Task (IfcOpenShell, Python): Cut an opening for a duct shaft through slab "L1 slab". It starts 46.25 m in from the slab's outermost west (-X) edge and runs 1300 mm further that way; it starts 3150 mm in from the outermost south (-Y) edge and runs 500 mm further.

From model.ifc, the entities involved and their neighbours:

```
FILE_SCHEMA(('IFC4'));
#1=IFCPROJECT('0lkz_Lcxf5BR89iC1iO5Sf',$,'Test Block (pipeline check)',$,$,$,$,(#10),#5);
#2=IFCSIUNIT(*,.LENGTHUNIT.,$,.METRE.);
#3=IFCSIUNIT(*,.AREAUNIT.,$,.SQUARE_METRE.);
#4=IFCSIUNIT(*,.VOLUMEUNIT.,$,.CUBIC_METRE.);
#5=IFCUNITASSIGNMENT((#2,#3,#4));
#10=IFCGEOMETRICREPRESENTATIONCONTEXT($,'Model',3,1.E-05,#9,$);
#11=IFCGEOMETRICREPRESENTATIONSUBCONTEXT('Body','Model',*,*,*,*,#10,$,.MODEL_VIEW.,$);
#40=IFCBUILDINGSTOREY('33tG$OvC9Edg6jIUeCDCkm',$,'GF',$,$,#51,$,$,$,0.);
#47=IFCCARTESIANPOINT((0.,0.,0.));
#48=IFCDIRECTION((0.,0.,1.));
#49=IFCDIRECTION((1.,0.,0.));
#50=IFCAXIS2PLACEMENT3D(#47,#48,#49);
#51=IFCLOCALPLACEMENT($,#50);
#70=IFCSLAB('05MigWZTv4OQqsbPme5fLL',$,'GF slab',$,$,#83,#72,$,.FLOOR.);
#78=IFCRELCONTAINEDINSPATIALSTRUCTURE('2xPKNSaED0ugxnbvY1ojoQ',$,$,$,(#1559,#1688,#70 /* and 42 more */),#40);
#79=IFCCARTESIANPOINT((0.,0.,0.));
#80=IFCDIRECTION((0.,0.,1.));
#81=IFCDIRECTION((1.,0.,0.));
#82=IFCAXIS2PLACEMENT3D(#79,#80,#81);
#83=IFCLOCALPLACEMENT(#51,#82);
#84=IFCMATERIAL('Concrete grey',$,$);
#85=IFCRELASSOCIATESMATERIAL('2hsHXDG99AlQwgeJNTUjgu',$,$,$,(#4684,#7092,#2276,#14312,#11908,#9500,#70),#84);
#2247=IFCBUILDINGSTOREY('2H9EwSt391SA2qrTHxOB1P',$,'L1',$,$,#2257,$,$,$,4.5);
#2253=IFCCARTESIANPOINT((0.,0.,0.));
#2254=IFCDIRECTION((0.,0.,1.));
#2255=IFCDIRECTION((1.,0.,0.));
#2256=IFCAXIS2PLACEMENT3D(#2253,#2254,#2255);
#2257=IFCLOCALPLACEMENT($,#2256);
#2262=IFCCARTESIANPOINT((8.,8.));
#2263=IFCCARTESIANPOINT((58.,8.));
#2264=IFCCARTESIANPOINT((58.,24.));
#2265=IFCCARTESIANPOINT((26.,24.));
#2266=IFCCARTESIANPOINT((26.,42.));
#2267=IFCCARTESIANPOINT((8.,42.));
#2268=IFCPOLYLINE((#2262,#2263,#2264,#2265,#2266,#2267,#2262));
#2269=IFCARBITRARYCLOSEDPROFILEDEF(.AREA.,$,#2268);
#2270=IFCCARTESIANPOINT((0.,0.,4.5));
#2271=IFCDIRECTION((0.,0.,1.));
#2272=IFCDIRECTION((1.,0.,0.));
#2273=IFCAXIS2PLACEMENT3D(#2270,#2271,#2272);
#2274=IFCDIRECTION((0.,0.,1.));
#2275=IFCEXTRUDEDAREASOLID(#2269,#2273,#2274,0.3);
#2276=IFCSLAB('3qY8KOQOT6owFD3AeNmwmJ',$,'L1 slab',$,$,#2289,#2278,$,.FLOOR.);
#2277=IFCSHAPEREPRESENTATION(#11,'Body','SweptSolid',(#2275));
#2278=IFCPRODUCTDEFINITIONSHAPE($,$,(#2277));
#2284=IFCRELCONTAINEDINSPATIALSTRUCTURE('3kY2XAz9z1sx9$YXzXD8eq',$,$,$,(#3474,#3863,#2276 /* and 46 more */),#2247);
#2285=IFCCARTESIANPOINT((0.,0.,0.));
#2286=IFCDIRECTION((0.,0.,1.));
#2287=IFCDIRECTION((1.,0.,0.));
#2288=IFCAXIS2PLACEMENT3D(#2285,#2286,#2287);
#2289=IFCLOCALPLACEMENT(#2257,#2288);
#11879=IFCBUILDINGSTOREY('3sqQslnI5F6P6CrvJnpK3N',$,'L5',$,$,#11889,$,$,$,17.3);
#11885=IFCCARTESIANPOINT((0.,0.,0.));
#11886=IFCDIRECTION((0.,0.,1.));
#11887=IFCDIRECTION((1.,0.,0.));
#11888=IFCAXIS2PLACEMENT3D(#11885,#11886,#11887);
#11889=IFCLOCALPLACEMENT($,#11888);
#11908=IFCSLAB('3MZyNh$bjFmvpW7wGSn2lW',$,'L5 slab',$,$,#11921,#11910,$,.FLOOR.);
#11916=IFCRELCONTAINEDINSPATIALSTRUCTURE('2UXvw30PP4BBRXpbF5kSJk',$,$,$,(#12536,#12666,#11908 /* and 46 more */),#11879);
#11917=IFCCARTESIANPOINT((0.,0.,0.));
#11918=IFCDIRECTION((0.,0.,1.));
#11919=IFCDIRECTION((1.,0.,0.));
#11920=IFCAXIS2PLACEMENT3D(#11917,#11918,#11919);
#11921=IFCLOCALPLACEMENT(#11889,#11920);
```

```python
import numpy as np
import ifcopenshell
import ifcopenshell.api.feature
import ifcopenshell.api.geometry
import ifcopenshell.api.root
import ifcopenshell.geom
import ifcopenshell.util.placement
import ifcopenshell.util.representation
import ifcopenshell.util.shape
import ifcopenshell.util.unit

model = ifcopenshell.open("model.ifc")
unit_scale = ifcopenshell.util.unit.calculate_unit_scale(model)
settings = ifcopenshell.geom.settings()


def volume(element):
    """Net volume in cubic metres, openings subtracted."""
    shape = ifcopenshell.geom.create_shape(settings, element)
    return ifcopenshell.util.shape.get_volume(shape.geometry)


slab = model.by_id(2276)
before = volume(slab)

# Extent in the slab's own axes, in metres. The edges named are its -X and -Y sides.
slab_shape = ifcopenshell.geom.create_shape(settings, slab)
vertices = ifcopenshell.util.shape.get_vertices(slab_shape.geometry)
x_min, y_min, bottom = vertices.min(axis=0)
top = vertices[:, 2].max()

opening = ifcopenshell.api.root.create_entity(model, ifc_class="IfcOpeningElement", name="Duct shaft opening", predefined_type="OPENING")
context = ifcopenshell.util.representation.get_context(model, "Model", "Body", "MODEL_VIEW")
width, depth = 1.3, 0.5
outline = [(0.0, 0.0), (width, 0.0), (width, depth), (0.0, depth), (0.0, 0.0)]
# Overshoot both faces by 50 mm so the cut is clean.
shape = ifcopenshell.api.geometry.add_slab_representation(
    model, context=context, depth=top - bottom + 0.1, polyline=outline
)
ifcopenshell.api.geometry.assign_representation(model, product=opening, representation=shape)

matrix = ifcopenshell.util.placement.get_local_placement(slab.ObjectPlacement)
matrix[:, 3] = matrix @ np.append(np.array([x_min + 46.25, y_min + 3.15, bottom - 0.05]) / unit_scale, 1.0)
ifcopenshell.api.geometry.edit_object_placement(model, product=opening, matrix=matrix, is_si=False)
ifcopenshell.api.feature.add_feature(model, feature=opening, element=slab)

after = volume(slab)

print(f"slab volume {before:.3f} -> {after:.3f} m3")

model.write("model_edited.ifc")
```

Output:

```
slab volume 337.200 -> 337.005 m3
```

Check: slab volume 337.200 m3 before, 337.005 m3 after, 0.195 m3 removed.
